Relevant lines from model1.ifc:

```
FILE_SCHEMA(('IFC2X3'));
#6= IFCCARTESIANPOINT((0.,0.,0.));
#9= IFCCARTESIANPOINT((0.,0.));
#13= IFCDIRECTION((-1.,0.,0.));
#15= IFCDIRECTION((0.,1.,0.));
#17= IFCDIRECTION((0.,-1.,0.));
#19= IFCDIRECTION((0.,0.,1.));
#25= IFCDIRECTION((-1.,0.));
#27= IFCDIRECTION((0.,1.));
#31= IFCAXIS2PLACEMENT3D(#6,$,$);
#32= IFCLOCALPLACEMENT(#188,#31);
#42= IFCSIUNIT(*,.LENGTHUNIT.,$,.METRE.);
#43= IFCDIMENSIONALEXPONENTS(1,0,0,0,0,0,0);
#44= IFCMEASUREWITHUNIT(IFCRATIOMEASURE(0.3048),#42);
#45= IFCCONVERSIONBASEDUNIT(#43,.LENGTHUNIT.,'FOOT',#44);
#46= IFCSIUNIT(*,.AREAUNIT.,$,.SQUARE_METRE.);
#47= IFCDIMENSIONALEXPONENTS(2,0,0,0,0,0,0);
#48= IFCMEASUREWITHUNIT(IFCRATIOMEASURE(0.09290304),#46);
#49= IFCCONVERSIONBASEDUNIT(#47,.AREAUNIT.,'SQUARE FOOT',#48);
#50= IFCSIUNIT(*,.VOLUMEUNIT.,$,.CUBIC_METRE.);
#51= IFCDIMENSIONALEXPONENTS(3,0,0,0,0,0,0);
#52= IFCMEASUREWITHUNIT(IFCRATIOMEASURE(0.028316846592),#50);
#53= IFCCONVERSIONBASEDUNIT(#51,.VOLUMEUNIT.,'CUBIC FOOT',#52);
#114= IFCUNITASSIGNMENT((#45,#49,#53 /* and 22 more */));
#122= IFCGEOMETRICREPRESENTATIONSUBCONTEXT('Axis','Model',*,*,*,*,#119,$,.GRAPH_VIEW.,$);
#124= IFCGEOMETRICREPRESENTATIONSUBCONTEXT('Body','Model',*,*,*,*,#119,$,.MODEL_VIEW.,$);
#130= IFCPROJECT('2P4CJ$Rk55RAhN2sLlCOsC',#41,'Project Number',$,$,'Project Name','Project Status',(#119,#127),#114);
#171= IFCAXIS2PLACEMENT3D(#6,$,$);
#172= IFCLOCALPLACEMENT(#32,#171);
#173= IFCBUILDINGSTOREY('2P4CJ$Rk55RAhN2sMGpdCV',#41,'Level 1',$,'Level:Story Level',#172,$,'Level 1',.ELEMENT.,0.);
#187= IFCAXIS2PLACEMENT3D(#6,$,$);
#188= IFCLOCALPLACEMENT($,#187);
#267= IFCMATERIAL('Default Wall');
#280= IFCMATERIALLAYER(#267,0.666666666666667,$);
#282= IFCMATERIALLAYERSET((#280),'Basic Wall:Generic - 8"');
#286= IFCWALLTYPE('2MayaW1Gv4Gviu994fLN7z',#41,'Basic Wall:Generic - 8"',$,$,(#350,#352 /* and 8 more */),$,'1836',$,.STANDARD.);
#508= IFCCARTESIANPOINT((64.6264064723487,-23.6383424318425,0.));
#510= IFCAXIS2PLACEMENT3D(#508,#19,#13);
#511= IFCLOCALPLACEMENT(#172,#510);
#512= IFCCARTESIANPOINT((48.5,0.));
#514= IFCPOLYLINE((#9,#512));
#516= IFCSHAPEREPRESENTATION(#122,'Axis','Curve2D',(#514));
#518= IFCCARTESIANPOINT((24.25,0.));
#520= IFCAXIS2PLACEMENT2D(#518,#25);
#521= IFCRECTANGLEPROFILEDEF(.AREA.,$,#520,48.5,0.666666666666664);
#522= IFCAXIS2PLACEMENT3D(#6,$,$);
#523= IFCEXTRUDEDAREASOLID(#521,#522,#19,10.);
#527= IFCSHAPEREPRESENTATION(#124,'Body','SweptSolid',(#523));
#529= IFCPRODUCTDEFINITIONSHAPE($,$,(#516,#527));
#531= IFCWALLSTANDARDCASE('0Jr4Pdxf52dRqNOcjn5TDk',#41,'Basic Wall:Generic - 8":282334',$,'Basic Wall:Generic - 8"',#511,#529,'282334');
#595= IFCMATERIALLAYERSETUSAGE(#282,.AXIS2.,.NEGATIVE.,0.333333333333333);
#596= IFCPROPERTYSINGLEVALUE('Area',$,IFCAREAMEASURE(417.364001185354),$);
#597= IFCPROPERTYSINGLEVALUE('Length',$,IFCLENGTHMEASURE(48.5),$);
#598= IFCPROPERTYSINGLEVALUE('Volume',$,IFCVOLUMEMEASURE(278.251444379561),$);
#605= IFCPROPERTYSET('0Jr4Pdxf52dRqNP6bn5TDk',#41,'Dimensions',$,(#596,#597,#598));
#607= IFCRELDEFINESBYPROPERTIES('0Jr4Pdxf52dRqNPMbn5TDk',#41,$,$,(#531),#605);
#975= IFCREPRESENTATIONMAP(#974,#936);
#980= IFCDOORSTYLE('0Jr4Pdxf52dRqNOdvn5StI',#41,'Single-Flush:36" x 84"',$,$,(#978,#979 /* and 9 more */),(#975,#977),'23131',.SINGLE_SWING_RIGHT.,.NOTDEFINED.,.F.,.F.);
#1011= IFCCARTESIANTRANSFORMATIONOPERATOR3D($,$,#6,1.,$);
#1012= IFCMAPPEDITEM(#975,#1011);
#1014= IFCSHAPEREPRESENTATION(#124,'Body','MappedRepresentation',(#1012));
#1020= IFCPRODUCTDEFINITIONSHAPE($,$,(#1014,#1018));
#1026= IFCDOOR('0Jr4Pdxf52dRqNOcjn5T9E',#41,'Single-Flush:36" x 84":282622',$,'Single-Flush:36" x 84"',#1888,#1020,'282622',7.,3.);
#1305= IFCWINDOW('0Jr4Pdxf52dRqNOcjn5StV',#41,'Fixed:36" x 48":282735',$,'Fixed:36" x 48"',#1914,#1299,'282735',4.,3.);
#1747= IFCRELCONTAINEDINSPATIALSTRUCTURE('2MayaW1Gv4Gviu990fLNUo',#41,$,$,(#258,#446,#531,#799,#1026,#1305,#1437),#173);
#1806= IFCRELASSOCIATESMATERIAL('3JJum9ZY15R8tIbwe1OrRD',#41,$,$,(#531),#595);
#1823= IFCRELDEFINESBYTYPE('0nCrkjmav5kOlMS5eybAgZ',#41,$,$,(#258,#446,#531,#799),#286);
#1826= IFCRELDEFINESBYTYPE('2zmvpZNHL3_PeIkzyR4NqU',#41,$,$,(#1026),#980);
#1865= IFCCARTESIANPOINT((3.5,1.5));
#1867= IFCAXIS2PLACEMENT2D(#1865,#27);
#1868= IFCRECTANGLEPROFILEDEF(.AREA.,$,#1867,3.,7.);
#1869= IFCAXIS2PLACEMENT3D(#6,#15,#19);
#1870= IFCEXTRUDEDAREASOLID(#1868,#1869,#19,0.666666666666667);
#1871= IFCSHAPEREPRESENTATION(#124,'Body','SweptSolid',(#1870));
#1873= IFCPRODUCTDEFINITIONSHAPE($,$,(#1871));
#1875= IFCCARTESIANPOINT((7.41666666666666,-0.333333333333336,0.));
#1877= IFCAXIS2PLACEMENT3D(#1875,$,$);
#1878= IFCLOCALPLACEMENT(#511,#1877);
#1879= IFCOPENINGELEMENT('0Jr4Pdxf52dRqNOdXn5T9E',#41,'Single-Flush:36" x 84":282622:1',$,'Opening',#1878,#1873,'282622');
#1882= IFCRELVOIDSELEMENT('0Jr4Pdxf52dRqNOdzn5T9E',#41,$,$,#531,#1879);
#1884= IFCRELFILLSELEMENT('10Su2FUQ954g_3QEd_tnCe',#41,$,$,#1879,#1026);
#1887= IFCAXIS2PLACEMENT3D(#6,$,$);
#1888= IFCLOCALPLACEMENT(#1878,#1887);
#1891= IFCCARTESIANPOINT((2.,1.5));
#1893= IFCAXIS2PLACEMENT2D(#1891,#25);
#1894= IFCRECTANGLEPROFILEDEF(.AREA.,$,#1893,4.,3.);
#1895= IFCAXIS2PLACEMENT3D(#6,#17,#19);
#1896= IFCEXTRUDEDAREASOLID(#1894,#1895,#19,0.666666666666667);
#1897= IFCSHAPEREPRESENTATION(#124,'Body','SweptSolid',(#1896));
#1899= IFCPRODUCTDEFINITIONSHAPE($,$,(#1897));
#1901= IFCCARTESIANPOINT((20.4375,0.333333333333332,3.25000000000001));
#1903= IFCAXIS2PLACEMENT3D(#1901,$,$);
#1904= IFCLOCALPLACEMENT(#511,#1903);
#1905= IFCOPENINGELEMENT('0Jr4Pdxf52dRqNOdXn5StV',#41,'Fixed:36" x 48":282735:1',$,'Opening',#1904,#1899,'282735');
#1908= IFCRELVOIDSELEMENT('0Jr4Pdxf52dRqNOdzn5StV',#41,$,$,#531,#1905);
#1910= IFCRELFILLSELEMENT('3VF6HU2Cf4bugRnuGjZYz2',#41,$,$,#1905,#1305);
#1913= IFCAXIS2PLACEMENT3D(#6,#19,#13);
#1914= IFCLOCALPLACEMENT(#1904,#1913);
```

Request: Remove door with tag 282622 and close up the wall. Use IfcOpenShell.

```python
import ifcopenshell
import ifcopenshell.api.feature
import ifcopenshell.api.pset
import ifcopenshell.api.root
import ifcopenshell.geom
import ifcopenshell.util.element
import ifcopenshell.util.shape
import ifcopenshell.util.unit

model = ifcopenshell.open("model1.ifc")
area_scale = ifcopenshell.util.unit.calculate_unit_scale(model, "AREAUNIT")
volume_scale = ifcopenshell.util.unit.calculate_unit_scale(model, "VOLUMEUNIT")
settings = ifcopenshell.geom.settings()


def volume(element):
    """Net volume in cubic metres, openings subtracted."""
    shape = ifcopenshell.geom.create_shape(settings, element)
    return ifcopenshell.util.shape.get_volume(shape.geometry)


door = model.by_id(1026)
opening = door.FillsVoids[0].RelatingOpeningElement
wall = opening.VoidsElements[0].RelatingBuildingElement
before = volume(wall)

ifcopenshell.api.root.remove_product(model, product=door)
ifcopenshell.api.feature.remove_feature(model, feature=opening)

after = volume(wall)
thickness = 0.2032  # wall thickness in metres

# Update the wall's stored quantities.
pset = model.by_id(ifcopenshell.util.element.get_pset(wall, "Dimensions", should_inherit=False)["id"])
ifcopenshell.api.pset.edit_pset(model, pset=pset, properties={
    "Area": model.create_entity("IfcAreaMeasure", after / thickness / area_scale),
    "Volume": model.create_entity("IfcVolumeMeasure", after / volume_scale),
})

print(f"wall volume {before:.3f} -> {after:.3f} m3")

model.write("model1_v2.ifc")
```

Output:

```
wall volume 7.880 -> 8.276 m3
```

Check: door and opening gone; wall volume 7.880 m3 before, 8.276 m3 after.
